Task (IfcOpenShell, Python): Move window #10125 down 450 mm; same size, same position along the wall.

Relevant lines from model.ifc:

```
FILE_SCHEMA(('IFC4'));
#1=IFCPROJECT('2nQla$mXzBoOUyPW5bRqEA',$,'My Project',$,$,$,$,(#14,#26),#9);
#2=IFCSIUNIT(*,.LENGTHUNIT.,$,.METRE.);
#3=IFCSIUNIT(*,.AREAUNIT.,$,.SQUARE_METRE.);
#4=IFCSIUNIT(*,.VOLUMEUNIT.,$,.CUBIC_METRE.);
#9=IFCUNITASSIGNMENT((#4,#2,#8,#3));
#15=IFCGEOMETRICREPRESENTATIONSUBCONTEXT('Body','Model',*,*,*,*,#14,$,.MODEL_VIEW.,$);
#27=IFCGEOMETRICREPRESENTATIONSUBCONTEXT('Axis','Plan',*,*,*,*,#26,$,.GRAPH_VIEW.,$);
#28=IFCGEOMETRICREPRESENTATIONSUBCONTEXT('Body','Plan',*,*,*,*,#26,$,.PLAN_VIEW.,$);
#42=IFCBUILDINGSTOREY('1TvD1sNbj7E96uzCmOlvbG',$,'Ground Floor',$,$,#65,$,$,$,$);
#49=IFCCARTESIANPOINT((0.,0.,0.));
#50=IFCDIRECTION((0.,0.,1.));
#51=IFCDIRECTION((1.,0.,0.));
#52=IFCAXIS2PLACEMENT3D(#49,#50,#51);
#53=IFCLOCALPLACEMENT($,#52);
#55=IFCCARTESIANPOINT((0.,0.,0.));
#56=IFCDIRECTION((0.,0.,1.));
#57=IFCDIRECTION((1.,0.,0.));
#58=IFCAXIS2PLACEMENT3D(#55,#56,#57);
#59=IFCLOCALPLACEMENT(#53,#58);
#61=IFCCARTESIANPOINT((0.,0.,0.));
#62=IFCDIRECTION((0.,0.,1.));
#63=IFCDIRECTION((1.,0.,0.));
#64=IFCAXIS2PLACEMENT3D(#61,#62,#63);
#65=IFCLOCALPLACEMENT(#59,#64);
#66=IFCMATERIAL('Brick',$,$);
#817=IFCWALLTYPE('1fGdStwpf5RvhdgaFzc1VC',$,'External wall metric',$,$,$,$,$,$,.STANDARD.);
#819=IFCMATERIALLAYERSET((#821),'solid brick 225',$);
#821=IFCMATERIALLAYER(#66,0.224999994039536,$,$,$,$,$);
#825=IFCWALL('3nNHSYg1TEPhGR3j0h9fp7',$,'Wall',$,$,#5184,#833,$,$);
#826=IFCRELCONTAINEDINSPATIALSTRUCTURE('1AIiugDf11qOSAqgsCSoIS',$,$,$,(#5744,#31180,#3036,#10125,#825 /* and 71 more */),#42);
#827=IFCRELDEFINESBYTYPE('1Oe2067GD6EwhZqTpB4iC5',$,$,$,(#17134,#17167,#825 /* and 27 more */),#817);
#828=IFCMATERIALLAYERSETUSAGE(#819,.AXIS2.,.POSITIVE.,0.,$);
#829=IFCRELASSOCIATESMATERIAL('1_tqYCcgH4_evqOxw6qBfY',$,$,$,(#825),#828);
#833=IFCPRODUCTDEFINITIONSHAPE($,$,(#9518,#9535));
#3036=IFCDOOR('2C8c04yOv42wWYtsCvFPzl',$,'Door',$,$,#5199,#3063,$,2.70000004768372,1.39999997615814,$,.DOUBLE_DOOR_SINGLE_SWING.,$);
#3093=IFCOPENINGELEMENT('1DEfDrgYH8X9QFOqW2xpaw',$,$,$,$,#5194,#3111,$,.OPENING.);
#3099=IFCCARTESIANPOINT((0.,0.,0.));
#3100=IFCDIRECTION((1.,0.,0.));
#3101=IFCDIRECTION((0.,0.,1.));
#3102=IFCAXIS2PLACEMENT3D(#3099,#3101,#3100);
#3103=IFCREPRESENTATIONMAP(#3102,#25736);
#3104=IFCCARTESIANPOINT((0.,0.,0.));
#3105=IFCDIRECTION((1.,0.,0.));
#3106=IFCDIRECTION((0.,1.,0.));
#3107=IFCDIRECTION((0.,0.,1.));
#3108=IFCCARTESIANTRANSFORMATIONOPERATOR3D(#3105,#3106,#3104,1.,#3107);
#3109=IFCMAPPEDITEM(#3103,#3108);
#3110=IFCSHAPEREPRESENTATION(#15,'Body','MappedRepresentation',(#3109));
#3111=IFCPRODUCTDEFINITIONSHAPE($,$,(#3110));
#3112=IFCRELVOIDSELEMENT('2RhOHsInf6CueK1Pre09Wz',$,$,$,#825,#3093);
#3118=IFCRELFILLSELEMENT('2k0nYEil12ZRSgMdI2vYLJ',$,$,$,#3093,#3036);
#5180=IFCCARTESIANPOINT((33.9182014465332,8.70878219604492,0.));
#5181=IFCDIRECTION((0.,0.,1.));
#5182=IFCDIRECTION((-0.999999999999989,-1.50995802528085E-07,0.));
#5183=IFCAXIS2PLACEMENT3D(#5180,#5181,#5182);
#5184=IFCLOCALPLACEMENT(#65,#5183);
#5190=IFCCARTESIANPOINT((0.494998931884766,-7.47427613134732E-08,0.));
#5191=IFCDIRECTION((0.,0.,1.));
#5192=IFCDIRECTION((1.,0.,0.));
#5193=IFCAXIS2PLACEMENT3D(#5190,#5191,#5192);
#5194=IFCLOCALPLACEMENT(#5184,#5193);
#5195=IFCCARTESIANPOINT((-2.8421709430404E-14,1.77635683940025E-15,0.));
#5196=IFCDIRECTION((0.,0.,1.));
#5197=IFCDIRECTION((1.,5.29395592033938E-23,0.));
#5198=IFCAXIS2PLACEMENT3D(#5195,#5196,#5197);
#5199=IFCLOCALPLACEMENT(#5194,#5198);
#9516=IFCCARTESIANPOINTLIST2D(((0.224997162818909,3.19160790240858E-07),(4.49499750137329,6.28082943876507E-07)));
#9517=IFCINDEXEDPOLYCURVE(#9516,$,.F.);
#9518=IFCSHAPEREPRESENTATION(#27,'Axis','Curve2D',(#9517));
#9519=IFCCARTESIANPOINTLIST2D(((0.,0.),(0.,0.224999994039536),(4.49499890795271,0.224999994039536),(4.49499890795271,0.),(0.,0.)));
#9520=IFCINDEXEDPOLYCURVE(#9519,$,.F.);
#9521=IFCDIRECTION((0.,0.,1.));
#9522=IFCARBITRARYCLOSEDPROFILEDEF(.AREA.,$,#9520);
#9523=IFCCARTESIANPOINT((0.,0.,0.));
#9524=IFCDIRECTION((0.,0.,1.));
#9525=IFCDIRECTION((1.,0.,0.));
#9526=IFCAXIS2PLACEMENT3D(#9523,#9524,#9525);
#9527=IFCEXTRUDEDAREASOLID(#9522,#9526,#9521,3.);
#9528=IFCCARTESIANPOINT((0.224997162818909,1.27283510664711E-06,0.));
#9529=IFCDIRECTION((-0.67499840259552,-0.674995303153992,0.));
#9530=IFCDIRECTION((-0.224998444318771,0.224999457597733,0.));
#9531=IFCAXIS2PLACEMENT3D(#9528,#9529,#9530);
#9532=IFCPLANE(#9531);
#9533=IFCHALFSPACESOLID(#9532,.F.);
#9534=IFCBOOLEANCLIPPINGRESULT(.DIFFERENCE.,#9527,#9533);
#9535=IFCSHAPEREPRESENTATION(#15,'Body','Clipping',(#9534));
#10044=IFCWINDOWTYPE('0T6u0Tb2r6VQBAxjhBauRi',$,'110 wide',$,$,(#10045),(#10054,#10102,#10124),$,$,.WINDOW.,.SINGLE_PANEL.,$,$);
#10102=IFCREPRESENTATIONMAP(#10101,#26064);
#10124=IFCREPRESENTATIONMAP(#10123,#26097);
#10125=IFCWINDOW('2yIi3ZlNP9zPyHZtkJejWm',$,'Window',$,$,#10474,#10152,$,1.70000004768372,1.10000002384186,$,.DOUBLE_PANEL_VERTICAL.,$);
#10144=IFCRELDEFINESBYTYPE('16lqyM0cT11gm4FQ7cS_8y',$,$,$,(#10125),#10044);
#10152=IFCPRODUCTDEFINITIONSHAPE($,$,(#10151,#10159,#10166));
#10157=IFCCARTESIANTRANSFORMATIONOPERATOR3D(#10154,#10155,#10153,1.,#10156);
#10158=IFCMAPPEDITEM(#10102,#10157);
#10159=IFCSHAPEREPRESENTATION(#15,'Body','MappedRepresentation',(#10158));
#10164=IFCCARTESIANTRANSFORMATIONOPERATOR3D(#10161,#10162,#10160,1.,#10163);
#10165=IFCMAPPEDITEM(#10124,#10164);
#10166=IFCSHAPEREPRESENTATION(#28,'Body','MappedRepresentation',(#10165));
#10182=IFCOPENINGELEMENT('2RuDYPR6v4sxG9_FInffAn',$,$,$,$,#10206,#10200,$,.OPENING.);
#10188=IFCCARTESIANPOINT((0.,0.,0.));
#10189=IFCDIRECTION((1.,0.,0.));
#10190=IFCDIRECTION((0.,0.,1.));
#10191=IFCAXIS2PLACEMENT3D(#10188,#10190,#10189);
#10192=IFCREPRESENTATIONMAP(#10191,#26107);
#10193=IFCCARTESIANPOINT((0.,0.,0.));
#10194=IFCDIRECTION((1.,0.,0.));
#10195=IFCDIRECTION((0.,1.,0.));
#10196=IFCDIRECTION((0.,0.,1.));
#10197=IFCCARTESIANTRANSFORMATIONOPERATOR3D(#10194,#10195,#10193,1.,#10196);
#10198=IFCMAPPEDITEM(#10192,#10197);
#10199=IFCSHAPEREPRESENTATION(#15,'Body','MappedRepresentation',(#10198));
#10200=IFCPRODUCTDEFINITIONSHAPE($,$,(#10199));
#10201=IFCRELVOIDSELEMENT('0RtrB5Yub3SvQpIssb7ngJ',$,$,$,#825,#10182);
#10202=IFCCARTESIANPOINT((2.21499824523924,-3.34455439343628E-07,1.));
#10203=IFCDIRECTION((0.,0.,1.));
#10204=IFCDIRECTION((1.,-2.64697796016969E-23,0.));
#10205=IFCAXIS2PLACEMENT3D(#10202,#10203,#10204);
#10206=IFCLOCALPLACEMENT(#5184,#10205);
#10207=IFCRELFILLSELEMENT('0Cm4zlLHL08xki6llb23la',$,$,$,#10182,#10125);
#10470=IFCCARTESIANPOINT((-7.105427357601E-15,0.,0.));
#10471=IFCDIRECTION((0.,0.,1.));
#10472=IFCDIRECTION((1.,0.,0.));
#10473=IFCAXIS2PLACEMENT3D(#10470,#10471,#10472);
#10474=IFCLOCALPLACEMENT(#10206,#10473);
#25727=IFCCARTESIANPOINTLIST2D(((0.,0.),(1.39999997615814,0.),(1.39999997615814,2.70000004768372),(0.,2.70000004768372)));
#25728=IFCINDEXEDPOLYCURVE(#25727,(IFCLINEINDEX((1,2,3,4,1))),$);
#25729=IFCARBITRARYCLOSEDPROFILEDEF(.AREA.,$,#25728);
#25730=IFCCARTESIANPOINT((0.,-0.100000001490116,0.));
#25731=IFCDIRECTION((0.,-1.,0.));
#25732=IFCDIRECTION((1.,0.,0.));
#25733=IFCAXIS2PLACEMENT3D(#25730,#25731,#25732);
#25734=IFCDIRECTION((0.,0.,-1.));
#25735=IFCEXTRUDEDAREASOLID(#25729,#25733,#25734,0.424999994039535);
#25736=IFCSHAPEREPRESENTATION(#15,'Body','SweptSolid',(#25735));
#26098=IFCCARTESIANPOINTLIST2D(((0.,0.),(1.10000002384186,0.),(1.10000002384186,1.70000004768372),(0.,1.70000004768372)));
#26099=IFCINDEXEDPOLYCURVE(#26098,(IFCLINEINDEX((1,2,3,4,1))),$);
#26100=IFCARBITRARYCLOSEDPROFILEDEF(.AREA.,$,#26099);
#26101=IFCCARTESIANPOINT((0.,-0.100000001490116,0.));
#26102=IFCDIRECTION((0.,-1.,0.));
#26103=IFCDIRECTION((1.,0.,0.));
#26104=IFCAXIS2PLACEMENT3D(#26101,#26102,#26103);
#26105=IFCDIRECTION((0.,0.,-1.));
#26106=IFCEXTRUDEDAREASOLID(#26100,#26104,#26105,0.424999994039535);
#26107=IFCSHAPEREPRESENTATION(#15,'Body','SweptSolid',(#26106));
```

```python
import numpy as np
import ifcopenshell
import ifcopenshell.api.geometry
import ifcopenshell.util.placement
import ifcopenshell.util.unit

model = ifcopenshell.open("model.ifc")
unit_scale = ifcopenshell.util.unit.calculate_unit_scale(model)

window = model.by_guid("2yIi3ZlNP9zPyHZtkJejWm")
opening = window.FillsVoids[0].RelatingOpeningElement
dz = -0.45

shift = np.array([0.0, 0.0, dz])
# The window is placed relative to its opening, so it follows when the opening moves.
matrix = ifcopenshell.util.placement.get_local_placement(opening.ObjectPlacement)
matrix[:3, 3] += shift
ifcopenshell.api.geometry.edit_object_placement(
    model, product=opening, matrix=matrix, is_si=False, should_transform_children=True
)

print(f"moved by {dz * unit_scale:+.3f} m")

model.write("model-out.ifc")
```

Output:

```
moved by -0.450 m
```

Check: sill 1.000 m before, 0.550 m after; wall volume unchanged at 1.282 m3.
